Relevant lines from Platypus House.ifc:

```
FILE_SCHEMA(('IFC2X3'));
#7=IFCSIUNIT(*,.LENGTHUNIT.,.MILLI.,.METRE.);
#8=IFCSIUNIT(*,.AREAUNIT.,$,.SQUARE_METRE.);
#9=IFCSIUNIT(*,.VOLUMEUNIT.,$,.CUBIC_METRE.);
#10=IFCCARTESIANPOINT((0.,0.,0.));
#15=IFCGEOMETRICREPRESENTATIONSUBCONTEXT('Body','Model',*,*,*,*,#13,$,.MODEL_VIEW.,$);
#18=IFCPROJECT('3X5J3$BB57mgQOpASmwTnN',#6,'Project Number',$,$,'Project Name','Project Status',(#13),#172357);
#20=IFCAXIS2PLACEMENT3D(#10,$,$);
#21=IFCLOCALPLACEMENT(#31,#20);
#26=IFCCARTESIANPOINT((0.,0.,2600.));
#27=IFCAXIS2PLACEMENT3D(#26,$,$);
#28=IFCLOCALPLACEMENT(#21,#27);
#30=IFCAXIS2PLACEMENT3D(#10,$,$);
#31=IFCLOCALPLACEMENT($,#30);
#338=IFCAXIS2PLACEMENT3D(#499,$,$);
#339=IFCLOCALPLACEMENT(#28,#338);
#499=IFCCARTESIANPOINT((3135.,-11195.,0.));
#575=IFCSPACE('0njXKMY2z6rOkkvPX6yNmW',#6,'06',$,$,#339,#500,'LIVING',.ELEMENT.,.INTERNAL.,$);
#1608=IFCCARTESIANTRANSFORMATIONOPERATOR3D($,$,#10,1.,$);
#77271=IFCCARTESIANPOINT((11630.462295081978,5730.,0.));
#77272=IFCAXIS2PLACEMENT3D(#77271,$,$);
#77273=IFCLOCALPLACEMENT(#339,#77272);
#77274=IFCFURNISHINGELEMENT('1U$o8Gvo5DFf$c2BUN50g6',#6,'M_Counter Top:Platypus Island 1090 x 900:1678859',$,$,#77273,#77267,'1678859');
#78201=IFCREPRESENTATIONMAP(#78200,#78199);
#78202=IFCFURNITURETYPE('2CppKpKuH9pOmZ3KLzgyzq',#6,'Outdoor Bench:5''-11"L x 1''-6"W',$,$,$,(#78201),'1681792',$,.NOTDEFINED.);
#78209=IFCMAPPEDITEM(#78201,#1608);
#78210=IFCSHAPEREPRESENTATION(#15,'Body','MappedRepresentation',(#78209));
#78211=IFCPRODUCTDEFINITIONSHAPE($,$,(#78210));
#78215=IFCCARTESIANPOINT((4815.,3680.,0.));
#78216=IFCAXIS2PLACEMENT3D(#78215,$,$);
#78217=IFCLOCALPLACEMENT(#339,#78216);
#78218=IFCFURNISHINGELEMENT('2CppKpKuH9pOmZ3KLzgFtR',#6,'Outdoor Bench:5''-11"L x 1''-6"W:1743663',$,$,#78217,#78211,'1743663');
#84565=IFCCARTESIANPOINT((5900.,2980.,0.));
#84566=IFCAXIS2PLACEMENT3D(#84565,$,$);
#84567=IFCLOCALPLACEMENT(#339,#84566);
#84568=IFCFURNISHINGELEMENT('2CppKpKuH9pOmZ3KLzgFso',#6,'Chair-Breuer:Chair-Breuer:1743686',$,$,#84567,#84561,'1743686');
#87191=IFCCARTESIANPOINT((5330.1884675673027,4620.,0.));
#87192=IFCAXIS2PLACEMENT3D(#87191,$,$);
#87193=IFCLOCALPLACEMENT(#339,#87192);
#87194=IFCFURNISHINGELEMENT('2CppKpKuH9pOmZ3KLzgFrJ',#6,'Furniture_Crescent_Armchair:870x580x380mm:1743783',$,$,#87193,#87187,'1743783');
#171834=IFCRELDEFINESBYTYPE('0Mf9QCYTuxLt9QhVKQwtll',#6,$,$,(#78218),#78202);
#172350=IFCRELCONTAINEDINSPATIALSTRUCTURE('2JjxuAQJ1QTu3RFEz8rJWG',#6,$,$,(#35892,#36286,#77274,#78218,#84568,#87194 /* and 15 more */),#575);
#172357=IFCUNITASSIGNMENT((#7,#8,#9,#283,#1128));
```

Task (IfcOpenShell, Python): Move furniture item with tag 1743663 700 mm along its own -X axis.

```python
import ifcopenshell
import ifcopenshell.api.geometry
import ifcopenshell.util.placement
import ifcopenshell.util.unit

model = ifcopenshell.open("Platypus House.ifc")
unit_scale = ifcopenshell.util.unit.calculate_unit_scale(model)

item = model.by_id(78218)
matrix = ifcopenshell.util.placement.get_local_placement(item.ObjectPlacement)
matrix[:3, 3] -= matrix[:3, 0] * 0.7 / unit_scale
ifcopenshell.api.geometry.edit_object_placement(model, product=item, matrix=matrix, is_si=False)

print(ifcopenshell.util.placement.get_local_placement(item.ObjectPlacement).round(3) + 0.0)

model.write("Platypus House_rev.ifc")
```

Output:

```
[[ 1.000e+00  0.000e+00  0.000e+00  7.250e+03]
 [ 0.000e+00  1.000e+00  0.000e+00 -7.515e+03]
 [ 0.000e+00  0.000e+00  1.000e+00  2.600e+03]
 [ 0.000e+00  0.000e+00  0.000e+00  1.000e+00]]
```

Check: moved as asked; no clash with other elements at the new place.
